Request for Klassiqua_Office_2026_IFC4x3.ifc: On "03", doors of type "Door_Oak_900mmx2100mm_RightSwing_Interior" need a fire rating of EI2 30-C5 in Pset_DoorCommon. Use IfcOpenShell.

First a look at what the model holds.

```python
import ifcopenshell
import ifcopenshell.util.element

model = ifcopenshell.open("Klassiqua_Office_2026_IFC4x3.ifc")
print(model.schema)
storey = next(s for s in model.by_type("IfcBuildingStorey") if s.Name == "03")
doors = [e for e in ifcopenshell.util.element.get_decomposition(storey) if e.is_a("IfcDoor")]
seen = {}
for e in doors:
    element_type = ifcopenshell.util.element.get_type(e)
    key = (element_type.Name if element_type != e and element_type else None, ifcopenshell.util.element.get_pset(e, "Pset_DoorCommon", "FireRating"))
    seen[key] = seen.get(key, 0) + 1
for (name, value), count in sorted(seen.items(), key=str):
    print(count, "x", name, "|", value)
```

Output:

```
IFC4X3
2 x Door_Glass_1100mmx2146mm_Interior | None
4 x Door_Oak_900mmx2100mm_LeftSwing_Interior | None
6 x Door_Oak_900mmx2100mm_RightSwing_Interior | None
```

```python
import ifcopenshell
import ifcopenshell.api.pset
import ifcopenshell.util.element

model = ifcopenshell.open("Klassiqua_Office_2026_IFC4x3.ifc")

storey = next(s for s in model.by_type("IfcBuildingStorey") if s.Name == "03")
doors = [e for e in ifcopenshell.util.element.get_decomposition(storey) if e.is_a("IfcDoor")]

count = 0
for e in doors:
    element_type = ifcopenshell.util.element.get_type(e)
    if element_type in (None, e) or element_type.Name != "Door_Oak_900mmx2100mm_RightSwing_Interior":
        continue
    # add_pset returns the element's existing set when there is one.
    pset = ifcopenshell.api.pset.add_pset(model, product=e, name="Pset_DoorCommon")
    ifcopenshell.api.pset.edit_pset(model, pset=pset, properties={"FireRating": "EI2 30-C5"})
    count += 1

print(count, "doors updated")

model.write("Klassiqua_Office_2026_IFC4x3_updated.ifc")
```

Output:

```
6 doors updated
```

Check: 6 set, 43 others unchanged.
